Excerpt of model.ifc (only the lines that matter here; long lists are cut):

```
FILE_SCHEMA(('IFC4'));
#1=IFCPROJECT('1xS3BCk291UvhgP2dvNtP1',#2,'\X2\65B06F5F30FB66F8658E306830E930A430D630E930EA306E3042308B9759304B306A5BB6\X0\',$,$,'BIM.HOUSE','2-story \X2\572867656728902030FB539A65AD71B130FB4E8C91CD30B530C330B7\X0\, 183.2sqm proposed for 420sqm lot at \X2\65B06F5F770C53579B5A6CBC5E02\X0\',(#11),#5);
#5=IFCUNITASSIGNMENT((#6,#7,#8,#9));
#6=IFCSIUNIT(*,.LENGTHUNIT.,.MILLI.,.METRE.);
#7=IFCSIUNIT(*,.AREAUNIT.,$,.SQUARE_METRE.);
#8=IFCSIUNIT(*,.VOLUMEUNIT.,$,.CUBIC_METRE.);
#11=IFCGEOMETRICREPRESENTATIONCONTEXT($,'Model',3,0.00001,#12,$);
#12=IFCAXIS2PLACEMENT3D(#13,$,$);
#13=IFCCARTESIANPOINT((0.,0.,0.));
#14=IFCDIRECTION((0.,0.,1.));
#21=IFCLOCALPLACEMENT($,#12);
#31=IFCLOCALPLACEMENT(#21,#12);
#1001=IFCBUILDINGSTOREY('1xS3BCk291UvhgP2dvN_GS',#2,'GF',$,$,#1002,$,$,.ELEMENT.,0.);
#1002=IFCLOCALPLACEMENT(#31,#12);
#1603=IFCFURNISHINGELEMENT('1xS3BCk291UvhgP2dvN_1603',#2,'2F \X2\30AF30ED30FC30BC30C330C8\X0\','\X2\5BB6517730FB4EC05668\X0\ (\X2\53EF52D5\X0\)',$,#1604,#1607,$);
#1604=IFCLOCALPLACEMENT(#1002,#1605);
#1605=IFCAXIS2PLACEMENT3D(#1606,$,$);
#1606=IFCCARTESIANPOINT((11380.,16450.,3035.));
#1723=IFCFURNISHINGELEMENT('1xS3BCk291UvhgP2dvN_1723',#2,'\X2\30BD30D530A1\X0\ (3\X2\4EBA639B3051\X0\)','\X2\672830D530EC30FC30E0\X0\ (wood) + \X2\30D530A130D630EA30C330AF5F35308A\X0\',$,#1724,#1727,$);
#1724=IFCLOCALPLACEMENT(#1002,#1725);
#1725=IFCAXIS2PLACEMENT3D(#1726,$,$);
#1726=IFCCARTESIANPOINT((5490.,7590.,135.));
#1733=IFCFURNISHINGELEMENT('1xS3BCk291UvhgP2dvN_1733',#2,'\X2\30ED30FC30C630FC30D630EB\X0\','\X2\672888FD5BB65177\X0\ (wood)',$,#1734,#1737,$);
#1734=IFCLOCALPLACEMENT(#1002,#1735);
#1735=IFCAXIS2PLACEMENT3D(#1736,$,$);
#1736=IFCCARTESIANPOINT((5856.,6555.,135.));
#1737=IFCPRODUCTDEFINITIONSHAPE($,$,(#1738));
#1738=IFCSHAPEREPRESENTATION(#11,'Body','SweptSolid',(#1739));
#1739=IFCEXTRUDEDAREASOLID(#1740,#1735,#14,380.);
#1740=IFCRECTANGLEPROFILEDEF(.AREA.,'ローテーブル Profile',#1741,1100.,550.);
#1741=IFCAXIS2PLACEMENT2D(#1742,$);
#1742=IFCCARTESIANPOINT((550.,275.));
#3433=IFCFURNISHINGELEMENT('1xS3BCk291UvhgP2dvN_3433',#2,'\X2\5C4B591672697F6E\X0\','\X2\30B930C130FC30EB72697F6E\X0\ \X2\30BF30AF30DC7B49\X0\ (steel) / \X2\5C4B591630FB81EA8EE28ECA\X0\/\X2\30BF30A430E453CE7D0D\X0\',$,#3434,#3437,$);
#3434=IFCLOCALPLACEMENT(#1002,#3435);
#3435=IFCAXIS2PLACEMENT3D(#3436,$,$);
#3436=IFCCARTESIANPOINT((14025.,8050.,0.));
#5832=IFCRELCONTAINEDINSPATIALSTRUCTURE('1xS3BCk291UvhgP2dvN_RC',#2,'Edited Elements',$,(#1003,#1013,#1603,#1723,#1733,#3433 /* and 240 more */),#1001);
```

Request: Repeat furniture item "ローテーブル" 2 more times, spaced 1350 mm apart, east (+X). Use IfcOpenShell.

```python
import numpy as np
import ifcopenshell
import ifcopenshell.api.geometry
import ifcopenshell.api.root
import ifcopenshell.util.element
import ifcopenshell.util.placement
import ifcopenshell.util.unit

model = ifcopenshell.open("model.ifc")
unit_scale = ifcopenshell.util.unit.calculate_unit_scale(model)


def reuse_history(source, copy):
    """copy_class also copies each property set's owner history, people and application; keep the originals."""
    for rel in copy.IsDefinedBy:
        if rel.is_a("IfcRelDefinesByProperties") and (history := rel.RelatingPropertyDefinition.OwnerHistory):
            rel.RelatingPropertyDefinition.OwnerHistory = source.OwnerHistory
            ifcopenshell.util.element.remove_deep2(model, history)


source = model.by_guid("1xS3BCk291UvhgP2dvN_1733")
base = ifcopenshell.util.placement.get_local_placement(source.ObjectPlacement)
step = np.array([1.0, 0.0, 0.0]) * 1.35 / unit_scale

for i in range(1, 3):
    copy = ifcopenshell.api.root.copy_class(model, product=source)
    copy.Representation = ifcopenshell.util.element.copy_deep(
        model, source.Representation, exclude=["IfcGeometricRepresentationContext", "IfcRepresentationMap"]
    )
    reuse_history(source, copy)
    matrix = base.copy()
    matrix[:3, 3] += i * step
    print("added at", matrix[:3, 3].round(3) + 0.0)
    ifcopenshell.api.geometry.edit_object_placement(model, product=copy, matrix=matrix, is_si=False)

model.write("model_rev.ifc")
```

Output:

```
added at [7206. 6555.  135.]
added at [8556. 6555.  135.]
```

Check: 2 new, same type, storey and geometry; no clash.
